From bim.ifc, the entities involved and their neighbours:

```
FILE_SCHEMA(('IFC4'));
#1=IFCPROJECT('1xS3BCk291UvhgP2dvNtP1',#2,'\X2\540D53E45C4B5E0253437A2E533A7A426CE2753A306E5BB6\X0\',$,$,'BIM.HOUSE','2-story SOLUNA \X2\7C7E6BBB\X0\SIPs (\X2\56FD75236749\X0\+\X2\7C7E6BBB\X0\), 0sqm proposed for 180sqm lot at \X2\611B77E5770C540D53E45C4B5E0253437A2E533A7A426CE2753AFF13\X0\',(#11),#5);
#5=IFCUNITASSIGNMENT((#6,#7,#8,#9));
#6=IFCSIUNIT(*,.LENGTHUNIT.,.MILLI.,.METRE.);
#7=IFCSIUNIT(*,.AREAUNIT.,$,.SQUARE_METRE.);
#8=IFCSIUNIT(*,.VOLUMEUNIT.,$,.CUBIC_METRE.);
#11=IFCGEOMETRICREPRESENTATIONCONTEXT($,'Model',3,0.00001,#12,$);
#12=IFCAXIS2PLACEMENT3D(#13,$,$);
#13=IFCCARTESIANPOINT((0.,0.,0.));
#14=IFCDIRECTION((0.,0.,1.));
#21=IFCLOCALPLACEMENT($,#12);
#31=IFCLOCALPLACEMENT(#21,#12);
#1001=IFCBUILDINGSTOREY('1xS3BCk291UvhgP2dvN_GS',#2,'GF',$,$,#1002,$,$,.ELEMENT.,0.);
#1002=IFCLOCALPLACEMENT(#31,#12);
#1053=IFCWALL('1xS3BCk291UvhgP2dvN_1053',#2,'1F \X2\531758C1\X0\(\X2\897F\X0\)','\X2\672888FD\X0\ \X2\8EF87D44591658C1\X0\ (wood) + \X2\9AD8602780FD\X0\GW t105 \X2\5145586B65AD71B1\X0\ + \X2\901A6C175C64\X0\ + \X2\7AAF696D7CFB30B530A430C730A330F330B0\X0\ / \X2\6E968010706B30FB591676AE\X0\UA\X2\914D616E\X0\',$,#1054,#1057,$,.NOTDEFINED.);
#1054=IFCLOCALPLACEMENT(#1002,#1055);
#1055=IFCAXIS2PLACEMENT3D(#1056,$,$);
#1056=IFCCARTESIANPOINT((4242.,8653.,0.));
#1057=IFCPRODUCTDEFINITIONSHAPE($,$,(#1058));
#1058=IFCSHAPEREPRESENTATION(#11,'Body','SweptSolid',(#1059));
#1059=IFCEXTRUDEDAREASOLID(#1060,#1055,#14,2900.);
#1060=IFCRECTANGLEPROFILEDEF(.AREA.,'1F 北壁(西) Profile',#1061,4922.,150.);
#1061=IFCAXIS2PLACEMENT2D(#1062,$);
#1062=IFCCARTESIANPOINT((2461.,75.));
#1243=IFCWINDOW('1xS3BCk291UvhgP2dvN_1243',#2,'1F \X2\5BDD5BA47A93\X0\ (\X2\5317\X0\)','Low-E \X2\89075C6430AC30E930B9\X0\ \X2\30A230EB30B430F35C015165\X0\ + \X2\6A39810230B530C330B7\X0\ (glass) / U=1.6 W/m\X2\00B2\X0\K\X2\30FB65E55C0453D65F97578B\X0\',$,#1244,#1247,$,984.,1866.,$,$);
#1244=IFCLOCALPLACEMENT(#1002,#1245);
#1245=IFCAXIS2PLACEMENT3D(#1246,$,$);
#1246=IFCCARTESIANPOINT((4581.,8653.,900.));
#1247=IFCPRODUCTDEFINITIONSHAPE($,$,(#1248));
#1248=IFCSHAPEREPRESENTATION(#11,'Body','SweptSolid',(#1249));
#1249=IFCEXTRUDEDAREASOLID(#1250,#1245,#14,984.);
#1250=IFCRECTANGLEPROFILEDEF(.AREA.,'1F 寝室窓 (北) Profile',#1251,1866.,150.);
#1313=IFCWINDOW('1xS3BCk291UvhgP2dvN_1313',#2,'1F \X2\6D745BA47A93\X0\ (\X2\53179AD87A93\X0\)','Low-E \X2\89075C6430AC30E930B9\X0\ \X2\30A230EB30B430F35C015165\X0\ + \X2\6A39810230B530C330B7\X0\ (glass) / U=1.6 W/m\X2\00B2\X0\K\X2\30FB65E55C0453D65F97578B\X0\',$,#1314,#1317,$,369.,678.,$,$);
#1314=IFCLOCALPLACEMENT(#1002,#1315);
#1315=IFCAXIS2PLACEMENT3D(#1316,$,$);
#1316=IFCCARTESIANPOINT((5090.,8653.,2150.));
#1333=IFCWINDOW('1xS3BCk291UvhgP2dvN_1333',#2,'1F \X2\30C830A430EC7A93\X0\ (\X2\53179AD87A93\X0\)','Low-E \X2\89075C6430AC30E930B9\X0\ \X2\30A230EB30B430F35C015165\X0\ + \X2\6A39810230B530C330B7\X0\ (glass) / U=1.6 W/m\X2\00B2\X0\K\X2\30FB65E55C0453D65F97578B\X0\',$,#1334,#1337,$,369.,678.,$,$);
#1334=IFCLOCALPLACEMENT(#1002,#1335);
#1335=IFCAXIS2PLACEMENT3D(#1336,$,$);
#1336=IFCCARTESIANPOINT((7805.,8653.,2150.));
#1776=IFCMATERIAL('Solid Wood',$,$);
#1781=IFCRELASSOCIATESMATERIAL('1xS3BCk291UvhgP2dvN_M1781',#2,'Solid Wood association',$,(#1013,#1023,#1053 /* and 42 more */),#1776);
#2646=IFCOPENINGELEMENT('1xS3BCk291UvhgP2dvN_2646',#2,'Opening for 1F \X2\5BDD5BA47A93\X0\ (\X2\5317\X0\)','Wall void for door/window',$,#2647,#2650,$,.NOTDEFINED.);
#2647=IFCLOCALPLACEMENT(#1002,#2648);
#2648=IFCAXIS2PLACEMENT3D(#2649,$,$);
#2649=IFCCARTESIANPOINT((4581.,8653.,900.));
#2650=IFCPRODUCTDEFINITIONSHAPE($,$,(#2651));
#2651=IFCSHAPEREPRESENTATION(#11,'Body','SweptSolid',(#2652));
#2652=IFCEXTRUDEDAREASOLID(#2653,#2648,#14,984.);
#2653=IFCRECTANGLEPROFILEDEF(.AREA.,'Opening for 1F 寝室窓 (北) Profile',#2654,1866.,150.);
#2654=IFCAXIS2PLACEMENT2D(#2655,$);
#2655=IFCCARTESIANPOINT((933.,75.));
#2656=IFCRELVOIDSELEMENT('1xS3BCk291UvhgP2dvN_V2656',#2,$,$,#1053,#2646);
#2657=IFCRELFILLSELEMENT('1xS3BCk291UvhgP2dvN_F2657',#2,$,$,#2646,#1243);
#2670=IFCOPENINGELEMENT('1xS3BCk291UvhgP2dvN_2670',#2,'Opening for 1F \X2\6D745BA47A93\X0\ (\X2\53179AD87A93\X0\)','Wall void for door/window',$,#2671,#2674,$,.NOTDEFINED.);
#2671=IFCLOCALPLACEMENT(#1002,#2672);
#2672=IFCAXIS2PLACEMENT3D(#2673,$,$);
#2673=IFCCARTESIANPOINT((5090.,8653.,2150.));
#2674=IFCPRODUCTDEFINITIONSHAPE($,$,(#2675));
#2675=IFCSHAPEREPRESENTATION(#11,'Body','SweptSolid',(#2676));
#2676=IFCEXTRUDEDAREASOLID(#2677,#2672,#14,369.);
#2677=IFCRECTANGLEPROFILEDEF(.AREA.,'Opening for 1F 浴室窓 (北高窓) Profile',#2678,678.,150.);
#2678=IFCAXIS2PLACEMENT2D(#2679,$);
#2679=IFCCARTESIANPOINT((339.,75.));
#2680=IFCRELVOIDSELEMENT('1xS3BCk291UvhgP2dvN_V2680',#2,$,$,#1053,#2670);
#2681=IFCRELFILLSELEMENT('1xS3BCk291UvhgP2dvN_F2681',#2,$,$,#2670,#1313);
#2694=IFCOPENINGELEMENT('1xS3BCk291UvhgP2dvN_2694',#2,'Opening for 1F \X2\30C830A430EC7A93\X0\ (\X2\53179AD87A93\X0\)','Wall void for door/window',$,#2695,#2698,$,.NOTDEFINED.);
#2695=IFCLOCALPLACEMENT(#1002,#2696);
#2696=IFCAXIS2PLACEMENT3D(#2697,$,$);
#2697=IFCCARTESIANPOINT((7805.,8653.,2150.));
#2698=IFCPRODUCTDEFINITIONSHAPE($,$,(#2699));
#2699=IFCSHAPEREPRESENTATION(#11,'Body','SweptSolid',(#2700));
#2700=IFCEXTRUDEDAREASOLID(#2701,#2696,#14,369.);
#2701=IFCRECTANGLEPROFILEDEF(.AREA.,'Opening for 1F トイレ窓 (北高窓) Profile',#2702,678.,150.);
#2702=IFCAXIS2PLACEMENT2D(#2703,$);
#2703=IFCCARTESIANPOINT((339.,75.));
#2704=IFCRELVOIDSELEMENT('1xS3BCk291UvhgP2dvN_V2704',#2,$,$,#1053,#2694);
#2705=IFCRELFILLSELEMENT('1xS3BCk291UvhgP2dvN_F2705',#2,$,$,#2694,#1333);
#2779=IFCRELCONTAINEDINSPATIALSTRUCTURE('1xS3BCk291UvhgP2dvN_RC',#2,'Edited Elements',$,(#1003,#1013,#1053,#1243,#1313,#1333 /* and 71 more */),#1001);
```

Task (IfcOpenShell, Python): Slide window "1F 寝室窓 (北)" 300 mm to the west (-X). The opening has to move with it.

```python
import ifcopenshell
import ifcopenshell.api.geometry
import ifcopenshell.util.placement

model = ifcopenshell.open("bim.ifc")

window = model.by_id(1243)
opening = window.FillsVoids[0].RelatingOpeningElement
wall = opening.VoidsElements[0].RelatingBuildingElement

wall_matrix = ifcopenshell.util.placement.get_local_placement(wall.ObjectPlacement)
shift = wall_matrix[:3, 0] * -300.0
before = ifcopenshell.util.placement.get_local_placement(window.ObjectPlacement)[:3, 3].copy()

# The window is not placed relative to its opening, so move both.
for product in (opening, window):
    matrix = ifcopenshell.util.placement.get_local_placement(product.ObjectPlacement)
    matrix[:3, 3] += shift
    ifcopenshell.api.geometry.edit_object_placement(model, product=product, matrix=matrix, is_si=False)

after = ifcopenshell.util.placement.get_local_placement(window.ObjectPlacement)[:3, 3]
print("window moved by", (after - before).round(3) + 0.0)

model.write("bim_edited.ifc")
```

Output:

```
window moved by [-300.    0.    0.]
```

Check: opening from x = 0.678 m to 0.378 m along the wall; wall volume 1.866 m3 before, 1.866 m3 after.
